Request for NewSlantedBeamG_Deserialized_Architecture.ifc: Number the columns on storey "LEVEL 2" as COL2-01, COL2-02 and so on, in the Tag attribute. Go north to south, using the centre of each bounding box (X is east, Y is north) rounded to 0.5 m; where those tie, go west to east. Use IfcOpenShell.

First a look at what the model holds.

```python
import ifcopenshell
import ifcopenshell.util.element
import ifcopenshell.util.placement

model = ifcopenshell.open("NewSlantedBeamG_Deserialized_Architecture.ifc")
print(model.schema)
storey = next(s for s in model.by_type("IfcBuildingStorey") if s.Name == "LEVEL 2")
columns = [e for e in ifcopenshell.util.element.get_decomposition(storey) if e.is_a("IfcColumn")]
for e in sorted(columns, key=lambda e: e.id()):
    origin = ifcopenshell.util.placement.get_local_placement(e.ObjectPlacement)[:3, 3]
    print(e.id(), e.Tag, e.Name, origin.round(2) + 0.0, sep=" | ")
```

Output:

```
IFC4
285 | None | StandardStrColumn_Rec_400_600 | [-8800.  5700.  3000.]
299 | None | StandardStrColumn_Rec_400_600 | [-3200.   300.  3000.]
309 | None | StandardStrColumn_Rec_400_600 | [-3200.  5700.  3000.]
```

```python
import ifcopenshell
import ifcopenshell.geom
import ifcopenshell.util.element
import ifcopenshell.util.shape

model = ifcopenshell.open("NewSlantedBeamG_Deserialized_Architecture.ifc")
settings = ifcopenshell.geom.settings()
settings.set("use-world-coords", True)


def centre(element):
    shape = ifcopenshell.geom.create_shape(settings, element)
    return ifcopenshell.util.shape.get_bbox_centroid(shape.geometry)


storey = next(s for s in model.by_type("IfcBuildingStorey") if s.Name == "LEVEL 2")
columns = [e for e in ifcopenshell.util.element.get_decomposition(storey) if e.is_a("IfcColumn")]

# Insertion points can sit at a corner or the storey origin, so sort by the geometry (in metres).
centres = {e: centre(e) for e in columns}
columns.sort(key=lambda e: (-round(centres[e][1] / 0.5), centres[e][0]))

for i, e in enumerate(columns, start=1):
    number = f"COL2-{i:02d}"
    e.Tag = number
    print(e.id(), number)

model.write("NewSlantedBeamG_Deserialized_Architecture_edited.ifc")
```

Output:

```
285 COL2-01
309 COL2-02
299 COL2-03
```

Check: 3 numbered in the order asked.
